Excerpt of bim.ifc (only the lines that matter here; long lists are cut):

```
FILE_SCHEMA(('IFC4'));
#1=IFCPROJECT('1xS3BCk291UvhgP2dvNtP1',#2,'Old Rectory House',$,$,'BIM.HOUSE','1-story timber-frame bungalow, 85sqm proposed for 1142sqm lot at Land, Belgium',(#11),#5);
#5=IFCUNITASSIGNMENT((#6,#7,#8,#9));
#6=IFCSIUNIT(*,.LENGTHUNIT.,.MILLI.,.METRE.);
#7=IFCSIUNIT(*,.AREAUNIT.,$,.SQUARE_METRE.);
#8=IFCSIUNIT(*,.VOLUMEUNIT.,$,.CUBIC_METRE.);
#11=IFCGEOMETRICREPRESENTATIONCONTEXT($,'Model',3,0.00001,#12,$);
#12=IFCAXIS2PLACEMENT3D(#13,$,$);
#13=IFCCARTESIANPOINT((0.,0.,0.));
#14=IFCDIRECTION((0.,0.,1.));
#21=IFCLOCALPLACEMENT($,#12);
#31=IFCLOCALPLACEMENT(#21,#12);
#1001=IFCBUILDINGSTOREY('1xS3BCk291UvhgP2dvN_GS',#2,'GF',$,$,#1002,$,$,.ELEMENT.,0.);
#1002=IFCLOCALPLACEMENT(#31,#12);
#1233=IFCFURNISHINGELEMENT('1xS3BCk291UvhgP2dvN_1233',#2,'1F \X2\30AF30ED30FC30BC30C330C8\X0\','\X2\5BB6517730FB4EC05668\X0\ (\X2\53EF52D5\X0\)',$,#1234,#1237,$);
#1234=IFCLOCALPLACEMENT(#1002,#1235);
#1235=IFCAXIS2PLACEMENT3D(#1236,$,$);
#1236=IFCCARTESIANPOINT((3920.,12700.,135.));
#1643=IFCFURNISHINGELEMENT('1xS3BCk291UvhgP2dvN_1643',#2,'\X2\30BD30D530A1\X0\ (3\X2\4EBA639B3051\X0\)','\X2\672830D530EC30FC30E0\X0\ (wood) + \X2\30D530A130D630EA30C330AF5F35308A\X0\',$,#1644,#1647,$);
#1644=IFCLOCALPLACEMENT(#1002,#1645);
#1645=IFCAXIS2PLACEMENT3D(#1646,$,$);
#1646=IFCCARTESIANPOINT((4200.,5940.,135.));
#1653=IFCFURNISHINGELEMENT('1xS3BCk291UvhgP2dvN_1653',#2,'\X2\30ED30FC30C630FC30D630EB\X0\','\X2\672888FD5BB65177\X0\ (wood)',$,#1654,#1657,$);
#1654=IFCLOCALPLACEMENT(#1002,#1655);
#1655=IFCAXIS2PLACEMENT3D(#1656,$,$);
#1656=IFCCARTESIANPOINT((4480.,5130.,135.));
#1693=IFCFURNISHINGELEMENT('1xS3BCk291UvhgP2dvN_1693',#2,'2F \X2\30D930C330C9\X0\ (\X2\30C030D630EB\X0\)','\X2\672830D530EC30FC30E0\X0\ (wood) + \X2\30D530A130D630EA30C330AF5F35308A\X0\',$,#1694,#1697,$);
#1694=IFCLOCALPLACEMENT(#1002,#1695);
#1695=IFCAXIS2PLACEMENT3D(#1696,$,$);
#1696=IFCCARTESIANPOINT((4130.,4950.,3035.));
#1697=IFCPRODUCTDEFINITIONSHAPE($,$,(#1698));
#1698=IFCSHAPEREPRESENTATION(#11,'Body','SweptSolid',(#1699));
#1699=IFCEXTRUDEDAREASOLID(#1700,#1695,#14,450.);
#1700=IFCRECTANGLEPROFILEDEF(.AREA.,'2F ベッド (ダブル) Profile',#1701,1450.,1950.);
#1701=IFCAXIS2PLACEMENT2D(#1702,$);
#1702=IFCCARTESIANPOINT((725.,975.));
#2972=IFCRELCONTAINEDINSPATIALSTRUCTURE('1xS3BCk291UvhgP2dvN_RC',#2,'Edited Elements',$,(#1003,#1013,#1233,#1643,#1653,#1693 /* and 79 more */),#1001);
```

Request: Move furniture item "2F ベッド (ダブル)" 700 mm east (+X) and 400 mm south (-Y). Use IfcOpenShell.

```python
import ifcopenshell
import ifcopenshell.api.geometry
import ifcopenshell.util.placement
import ifcopenshell.util.unit

model = ifcopenshell.open("bim.ifc")
unit_scale = ifcopenshell.util.unit.calculate_unit_scale(model)

item = model.by_guid("1xS3BCk291UvhgP2dvN_1693")
matrix = ifcopenshell.util.placement.get_local_placement(item.ObjectPlacement)
matrix[0, 3] += 0.7 / unit_scale
matrix[1, 3] -= 0.4 / unit_scale
ifcopenshell.api.geometry.edit_object_placement(model, product=item, matrix=matrix, is_si=False)

print(ifcopenshell.util.placement.get_local_placement(item.ObjectPlacement).round(3) + 0.0)

model.write("bim_edited.ifc")
```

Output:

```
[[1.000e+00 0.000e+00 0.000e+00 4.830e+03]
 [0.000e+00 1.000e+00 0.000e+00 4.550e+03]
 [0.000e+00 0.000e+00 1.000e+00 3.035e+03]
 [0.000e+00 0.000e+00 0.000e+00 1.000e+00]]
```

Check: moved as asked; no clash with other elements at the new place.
